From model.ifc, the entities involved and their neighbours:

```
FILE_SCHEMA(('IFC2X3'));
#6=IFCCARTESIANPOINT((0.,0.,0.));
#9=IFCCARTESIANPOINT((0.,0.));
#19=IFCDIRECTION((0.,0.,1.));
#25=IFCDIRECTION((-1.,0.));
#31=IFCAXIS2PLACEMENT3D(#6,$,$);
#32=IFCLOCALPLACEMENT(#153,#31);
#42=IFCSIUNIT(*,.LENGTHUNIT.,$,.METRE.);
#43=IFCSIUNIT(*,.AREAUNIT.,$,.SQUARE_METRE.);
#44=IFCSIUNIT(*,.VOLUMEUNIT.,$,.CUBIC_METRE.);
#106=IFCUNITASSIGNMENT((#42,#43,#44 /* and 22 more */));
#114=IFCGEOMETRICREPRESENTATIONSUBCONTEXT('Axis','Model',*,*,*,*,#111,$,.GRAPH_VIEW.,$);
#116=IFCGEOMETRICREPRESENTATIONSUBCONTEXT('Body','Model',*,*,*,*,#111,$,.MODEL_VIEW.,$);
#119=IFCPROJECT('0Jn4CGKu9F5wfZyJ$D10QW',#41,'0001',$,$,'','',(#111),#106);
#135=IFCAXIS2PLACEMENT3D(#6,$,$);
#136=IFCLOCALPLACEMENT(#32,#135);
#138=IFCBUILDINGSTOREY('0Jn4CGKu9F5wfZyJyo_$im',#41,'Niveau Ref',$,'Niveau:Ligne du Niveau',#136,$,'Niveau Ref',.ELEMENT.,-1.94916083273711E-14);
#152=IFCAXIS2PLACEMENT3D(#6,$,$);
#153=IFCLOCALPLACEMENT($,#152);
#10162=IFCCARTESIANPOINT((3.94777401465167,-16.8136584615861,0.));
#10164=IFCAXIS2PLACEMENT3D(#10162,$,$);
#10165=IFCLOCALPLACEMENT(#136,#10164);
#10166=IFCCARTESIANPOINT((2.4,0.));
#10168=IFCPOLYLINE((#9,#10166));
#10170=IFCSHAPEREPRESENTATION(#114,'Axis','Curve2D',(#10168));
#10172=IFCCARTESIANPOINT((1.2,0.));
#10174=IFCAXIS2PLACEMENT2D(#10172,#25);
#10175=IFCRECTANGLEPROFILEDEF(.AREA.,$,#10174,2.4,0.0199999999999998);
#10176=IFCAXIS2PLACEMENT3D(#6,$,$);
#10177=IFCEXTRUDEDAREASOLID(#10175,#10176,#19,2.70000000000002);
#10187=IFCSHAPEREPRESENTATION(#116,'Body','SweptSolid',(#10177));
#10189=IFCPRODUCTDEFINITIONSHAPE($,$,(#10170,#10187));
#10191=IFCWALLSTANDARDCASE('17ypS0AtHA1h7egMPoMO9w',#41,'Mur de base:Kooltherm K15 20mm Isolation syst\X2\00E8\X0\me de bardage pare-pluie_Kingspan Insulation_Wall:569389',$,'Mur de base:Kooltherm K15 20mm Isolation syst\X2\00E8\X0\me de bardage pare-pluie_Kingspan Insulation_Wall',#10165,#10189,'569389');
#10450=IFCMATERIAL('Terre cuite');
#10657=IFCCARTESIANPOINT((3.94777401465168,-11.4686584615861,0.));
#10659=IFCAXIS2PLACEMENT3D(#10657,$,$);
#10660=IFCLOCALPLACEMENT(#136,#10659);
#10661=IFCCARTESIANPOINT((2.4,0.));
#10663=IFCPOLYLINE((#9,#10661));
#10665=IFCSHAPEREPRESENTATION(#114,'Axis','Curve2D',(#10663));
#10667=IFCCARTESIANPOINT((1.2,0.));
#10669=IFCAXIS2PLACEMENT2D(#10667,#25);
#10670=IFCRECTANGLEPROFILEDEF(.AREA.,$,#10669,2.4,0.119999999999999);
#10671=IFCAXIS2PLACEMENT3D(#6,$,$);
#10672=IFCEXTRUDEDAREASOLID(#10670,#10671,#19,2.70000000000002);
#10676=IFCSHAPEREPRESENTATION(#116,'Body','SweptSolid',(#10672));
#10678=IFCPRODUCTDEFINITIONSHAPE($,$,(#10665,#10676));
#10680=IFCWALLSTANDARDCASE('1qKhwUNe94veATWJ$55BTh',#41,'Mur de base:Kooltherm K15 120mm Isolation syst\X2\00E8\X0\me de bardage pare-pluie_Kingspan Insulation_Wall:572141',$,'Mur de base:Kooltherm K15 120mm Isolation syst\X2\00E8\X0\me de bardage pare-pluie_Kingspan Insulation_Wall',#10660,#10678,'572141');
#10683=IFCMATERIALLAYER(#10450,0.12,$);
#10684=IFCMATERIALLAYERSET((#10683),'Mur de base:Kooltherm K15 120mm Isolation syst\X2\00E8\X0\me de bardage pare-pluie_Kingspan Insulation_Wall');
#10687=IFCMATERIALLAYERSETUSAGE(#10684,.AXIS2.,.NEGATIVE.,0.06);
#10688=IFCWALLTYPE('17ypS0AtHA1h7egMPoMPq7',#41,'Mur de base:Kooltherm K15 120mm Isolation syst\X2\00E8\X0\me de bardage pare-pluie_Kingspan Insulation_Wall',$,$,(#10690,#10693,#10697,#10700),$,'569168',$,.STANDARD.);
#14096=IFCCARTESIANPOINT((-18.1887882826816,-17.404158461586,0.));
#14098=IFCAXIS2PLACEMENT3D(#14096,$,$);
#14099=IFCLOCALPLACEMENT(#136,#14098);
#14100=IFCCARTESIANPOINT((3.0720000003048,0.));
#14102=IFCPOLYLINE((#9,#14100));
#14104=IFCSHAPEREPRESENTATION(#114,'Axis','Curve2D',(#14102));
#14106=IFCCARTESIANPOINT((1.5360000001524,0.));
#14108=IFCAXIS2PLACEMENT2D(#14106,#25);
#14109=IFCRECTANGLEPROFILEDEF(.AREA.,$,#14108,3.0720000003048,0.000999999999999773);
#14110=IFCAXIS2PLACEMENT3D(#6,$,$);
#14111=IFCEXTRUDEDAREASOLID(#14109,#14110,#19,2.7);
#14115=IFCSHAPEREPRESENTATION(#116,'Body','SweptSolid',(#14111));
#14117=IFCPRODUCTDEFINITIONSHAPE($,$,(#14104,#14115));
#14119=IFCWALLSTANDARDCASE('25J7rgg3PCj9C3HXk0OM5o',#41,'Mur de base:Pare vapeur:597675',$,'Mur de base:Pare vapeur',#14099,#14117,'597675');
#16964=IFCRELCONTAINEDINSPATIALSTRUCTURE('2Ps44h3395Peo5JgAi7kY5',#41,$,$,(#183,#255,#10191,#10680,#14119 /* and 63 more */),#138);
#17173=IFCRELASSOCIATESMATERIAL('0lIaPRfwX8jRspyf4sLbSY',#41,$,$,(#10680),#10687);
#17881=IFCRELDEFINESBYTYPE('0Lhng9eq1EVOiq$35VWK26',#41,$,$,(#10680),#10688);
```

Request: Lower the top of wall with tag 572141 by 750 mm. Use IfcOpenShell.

```python
import ifcopenshell
import ifcopenshell.geom
import ifcopenshell.util.representation
import ifcopenshell.util.shape

model = ifcopenshell.open("model.ifc")
settings = ifcopenshell.geom.settings()


def volume(element):
    """Net volume in cubic metres, openings subtracted."""
    shape = ifcopenshell.geom.create_shape(settings, element)
    return ifcopenshell.util.shape.get_volume(shape.geometry)


wall = model.by_id(10680)
before = volume(wall)

body = ifcopenshell.util.representation.get_representation(wall, "Model", "Body")
solid = body.Items[0]
old_height = solid.Depth
solid.Depth -= 0.75
after = volume(wall)

print(f"height {old_height:g} -> {solid.Depth:g}, volume {before:.3f} -> {after:.3f} m3")

model.write("model_updated.ifc")
```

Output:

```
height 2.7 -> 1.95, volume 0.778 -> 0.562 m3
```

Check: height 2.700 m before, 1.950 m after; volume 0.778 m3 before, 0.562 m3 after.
